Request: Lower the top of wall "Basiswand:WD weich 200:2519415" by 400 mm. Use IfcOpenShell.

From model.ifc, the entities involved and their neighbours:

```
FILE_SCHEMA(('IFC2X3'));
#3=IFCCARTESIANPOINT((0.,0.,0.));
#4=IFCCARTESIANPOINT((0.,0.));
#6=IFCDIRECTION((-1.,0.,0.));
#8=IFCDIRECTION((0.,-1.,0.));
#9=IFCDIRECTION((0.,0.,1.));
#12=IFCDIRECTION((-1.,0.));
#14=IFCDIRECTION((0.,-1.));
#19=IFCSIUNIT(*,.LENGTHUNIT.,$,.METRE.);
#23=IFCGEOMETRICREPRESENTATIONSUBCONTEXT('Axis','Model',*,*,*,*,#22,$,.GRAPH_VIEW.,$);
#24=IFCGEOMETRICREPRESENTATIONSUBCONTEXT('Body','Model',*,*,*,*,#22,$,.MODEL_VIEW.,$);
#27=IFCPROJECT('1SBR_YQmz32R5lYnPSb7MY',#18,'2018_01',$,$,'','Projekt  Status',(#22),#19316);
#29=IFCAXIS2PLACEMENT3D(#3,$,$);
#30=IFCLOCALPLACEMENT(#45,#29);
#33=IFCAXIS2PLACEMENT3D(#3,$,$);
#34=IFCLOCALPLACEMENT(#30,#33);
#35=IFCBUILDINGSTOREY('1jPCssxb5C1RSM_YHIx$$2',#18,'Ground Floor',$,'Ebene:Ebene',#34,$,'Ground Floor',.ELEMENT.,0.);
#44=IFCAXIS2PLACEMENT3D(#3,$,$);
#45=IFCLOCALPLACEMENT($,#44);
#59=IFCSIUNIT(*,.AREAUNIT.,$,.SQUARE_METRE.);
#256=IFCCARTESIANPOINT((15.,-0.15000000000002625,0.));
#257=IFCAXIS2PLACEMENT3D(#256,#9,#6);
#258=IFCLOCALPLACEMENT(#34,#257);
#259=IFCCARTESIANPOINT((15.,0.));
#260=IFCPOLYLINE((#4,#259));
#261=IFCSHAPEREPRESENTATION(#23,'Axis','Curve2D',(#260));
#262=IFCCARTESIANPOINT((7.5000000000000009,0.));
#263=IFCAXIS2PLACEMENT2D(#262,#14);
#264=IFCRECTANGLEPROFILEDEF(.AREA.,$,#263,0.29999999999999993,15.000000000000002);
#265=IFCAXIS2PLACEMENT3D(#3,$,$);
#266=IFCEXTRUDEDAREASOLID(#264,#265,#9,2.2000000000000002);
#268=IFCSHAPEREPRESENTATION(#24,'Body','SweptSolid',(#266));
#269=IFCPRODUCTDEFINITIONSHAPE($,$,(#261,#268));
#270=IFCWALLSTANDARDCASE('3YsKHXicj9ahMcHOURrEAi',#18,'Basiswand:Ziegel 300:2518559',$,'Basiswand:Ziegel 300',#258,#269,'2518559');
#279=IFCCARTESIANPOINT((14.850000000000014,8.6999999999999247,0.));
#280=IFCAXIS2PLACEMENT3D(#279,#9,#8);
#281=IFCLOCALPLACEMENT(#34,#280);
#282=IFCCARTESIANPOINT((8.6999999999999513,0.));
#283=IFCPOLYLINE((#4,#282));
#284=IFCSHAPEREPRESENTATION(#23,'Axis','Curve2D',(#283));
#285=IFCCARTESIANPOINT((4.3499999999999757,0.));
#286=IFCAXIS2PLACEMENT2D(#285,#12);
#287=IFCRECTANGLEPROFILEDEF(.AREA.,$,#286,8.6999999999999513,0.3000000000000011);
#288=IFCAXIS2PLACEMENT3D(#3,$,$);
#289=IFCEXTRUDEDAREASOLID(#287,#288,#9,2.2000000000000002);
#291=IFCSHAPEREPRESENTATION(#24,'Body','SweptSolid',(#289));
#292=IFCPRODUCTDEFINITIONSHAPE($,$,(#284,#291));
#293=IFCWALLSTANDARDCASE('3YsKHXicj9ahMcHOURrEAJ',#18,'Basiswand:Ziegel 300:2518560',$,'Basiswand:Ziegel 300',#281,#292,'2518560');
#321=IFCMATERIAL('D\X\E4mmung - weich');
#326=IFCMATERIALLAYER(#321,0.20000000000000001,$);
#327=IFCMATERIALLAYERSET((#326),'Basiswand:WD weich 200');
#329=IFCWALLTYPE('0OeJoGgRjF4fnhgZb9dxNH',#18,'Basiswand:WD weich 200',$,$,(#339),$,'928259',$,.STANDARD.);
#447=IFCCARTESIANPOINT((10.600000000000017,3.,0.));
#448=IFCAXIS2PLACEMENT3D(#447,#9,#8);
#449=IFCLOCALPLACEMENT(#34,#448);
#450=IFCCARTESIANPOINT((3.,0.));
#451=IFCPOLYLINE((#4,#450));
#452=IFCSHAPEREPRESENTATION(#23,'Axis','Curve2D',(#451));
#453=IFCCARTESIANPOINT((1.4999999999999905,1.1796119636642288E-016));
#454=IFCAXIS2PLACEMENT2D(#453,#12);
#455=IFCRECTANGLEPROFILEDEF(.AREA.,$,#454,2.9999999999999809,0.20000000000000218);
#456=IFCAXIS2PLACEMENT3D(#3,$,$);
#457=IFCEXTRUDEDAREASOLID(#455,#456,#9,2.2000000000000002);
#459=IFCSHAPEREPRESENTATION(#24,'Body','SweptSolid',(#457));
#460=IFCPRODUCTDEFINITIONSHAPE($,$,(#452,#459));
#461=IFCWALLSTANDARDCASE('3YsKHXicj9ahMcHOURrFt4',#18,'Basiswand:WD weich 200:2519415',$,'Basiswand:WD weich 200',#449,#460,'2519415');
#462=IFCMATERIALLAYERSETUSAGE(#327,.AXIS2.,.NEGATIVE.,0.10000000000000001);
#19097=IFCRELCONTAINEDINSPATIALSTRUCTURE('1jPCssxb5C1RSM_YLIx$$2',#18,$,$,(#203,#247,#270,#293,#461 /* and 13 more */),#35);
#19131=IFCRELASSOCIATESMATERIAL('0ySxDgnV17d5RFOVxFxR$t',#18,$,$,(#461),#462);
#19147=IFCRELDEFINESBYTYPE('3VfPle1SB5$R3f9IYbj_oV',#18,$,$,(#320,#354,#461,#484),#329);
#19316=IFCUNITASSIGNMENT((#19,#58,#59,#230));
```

```python
import ifcopenshell
import ifcopenshell.geom
import ifcopenshell.util.representation
import ifcopenshell.util.shape
import ifcopenshell.util.unit

model = ifcopenshell.open("model.ifc")
unit_scale = ifcopenshell.util.unit.calculate_unit_scale(model)
settings = ifcopenshell.geom.settings()


def volume(element):
    """Net volume in cubic metres, openings subtracted."""
    shape = ifcopenshell.geom.create_shape(settings, element)
    return ifcopenshell.util.shape.get_volume(shape.geometry)


wall = model.by_guid("3YsKHXicj9ahMcHOURrFt4")
before = volume(wall)

body = ifcopenshell.util.representation.get_representation(wall, "Model", "Body")
solid = body.Items[0]
old_height = solid.Depth
solid.Depth -= 0.4 / unit_scale
after = volume(wall)

print(f"height {old_height:g} -> {solid.Depth:g}, volume {before:.3f} -> {after:.3f} m3")

model.write("model-out.ifc")
```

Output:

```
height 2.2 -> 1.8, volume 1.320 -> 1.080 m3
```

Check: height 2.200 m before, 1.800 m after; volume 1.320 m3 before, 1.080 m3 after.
